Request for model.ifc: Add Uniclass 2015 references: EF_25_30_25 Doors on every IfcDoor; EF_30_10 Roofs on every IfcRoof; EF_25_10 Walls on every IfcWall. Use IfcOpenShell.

First a look at what the model holds.

```python
import ifcopenshell

model = ifcopenshell.open("model.ifc")
print(model.schema)
print("classifications:", [c.Name for c in model.by_type("IfcClassification")])
for ifc_class in ("IfcDoor", "IfcRoof", "IfcStair", "IfcWall", "IfcWindow"):
    print(ifc_class, len(model.by_type(ifc_class)))
```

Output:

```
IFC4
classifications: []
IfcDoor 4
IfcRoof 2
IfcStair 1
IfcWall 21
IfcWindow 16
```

```python
import ifcopenshell
import ifcopenshell.api.classification

model = ifcopenshell.open("model.ifc")

system = ifcopenshell.api.classification.add_classification(model, classification="Uniclass 2015")

codes = {
    "IfcDoor": ("EF_25_30_25", "Doors"),
    "IfcRoof": ("EF_30_10", "Roofs"),
    "IfcWall": ("EF_25_10", "Walls"),
}
for ifc_class, (code, name) in codes.items():
    products = model.by_type(ifc_class)
    ifcopenshell.api.classification.add_reference(
        model, products=products, classification=system, identification=code, name=name
    )
    print(code, len(products))

model.write("model_edited.ifc")
```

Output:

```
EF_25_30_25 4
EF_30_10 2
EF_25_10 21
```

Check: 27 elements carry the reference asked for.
